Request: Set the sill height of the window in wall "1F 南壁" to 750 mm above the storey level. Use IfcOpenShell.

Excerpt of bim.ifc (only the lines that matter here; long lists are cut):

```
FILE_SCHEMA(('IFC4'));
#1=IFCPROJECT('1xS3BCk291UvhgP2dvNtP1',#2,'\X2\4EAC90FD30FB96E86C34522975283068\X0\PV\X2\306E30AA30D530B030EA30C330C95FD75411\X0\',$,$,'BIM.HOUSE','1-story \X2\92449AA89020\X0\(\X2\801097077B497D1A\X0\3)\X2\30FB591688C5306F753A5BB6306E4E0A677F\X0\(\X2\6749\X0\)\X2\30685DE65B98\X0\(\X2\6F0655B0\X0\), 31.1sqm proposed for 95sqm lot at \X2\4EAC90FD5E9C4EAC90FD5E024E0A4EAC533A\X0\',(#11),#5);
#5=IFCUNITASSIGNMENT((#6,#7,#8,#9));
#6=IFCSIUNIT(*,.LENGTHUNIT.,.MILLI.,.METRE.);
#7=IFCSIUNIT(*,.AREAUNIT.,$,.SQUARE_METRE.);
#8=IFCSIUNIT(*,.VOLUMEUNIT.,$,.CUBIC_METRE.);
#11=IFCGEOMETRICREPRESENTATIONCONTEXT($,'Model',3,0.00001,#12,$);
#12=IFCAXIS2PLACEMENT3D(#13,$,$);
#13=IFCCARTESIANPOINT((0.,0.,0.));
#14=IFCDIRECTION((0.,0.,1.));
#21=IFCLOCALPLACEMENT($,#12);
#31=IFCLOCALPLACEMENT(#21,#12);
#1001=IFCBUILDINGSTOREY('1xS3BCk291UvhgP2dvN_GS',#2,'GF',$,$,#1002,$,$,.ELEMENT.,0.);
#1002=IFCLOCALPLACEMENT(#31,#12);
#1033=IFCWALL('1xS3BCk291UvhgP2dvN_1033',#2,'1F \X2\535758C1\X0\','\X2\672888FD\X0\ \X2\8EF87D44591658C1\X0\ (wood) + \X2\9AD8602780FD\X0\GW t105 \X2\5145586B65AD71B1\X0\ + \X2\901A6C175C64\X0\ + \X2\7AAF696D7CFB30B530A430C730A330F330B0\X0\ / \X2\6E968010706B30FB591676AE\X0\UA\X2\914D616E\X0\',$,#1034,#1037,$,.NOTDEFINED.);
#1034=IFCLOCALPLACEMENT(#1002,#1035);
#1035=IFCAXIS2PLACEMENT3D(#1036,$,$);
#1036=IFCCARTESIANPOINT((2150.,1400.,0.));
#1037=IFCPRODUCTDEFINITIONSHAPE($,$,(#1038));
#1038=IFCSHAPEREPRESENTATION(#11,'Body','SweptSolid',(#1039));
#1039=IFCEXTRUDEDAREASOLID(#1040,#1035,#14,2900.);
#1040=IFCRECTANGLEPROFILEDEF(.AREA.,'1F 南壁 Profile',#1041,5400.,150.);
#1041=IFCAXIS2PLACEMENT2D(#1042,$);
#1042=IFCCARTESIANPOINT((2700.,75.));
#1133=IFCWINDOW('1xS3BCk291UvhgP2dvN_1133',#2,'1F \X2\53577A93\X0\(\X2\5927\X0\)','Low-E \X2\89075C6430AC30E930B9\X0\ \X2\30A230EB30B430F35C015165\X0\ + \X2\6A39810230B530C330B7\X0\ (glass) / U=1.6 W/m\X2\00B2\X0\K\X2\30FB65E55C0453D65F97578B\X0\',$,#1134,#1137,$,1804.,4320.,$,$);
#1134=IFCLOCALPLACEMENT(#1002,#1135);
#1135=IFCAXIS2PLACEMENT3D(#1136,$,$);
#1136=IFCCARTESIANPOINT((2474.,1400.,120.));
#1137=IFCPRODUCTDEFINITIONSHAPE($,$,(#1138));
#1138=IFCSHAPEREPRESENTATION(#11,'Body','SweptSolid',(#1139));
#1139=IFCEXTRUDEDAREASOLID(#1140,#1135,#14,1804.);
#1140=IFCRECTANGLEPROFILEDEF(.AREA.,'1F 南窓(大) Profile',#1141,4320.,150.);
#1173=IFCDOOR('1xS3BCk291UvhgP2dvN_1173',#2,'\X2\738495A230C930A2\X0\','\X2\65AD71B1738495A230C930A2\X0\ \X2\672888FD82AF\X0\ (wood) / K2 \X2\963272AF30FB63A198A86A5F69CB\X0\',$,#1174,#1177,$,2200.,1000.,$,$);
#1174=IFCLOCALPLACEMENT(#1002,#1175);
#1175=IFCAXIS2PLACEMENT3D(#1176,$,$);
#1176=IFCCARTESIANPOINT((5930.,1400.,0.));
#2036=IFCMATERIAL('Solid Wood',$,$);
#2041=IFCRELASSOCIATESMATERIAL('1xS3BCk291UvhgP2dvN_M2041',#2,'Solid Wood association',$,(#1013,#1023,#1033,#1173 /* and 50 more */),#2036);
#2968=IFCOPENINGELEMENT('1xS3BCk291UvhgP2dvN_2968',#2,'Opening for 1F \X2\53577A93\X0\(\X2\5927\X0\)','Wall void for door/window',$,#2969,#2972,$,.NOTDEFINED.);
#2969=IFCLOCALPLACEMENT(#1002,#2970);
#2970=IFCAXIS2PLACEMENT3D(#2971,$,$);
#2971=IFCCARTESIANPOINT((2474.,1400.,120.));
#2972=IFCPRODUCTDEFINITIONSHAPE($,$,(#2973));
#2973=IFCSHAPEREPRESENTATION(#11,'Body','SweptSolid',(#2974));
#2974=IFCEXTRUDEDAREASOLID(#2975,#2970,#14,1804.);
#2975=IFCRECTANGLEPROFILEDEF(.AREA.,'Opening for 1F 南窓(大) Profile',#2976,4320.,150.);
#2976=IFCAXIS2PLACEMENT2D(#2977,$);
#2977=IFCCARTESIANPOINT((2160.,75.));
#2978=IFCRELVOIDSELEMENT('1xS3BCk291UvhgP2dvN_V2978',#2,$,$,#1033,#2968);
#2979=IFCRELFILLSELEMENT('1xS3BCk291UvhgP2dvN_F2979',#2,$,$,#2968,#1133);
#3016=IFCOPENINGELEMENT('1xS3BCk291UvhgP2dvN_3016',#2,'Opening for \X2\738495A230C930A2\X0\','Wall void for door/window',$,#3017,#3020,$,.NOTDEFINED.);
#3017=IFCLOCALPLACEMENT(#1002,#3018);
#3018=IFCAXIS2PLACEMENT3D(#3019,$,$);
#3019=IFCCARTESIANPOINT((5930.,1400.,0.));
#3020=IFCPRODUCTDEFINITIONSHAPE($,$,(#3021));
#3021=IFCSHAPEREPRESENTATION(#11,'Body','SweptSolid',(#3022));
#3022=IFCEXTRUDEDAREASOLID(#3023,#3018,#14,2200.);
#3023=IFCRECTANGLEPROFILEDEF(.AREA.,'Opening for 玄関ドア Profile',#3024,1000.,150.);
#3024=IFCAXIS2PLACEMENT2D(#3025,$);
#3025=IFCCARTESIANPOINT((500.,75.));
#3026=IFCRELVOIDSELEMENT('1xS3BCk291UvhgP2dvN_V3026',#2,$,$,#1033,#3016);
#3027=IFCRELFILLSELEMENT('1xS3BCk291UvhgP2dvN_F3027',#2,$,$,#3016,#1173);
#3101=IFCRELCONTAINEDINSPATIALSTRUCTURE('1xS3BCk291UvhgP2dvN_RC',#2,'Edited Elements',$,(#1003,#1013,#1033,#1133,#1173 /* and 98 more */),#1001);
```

```python
import numpy as np
import ifcopenshell
import ifcopenshell.api.geometry
import ifcopenshell.geom
import ifcopenshell.util.element
import ifcopenshell.util.placement
import ifcopenshell.util.shape
import ifcopenshell.util.unit

model = ifcopenshell.open("bim.ifc")
unit_scale = ifcopenshell.util.unit.calculate_unit_scale(model)

window = model.by_id(1133)
opening = window.FillsVoids[0].RelatingOpeningElement
storey = ifcopenshell.util.element.get_container(window, ifc_class="IfcBuildingStorey")
level = ifcopenshell.util.placement.get_local_placement(storey.ObjectPlacement)[2, 3]

# The opening's origin need not be at the sill, so measure its lowest point.
shape = ifcopenshell.geom.create_shape(ifcopenshell.geom.settings(), opening)
bottom = ifcopenshell.util.shape.get_shape_bottom_elevation(shape, shape.geometry) / unit_scale
dz = level + 0.75 / unit_scale - bottom

shift = np.array([0.0, 0.0, dz])
# The window is not placed relative to its opening, so move both.
for product in (opening, window):
    matrix = ifcopenshell.util.placement.get_local_placement(product.ObjectPlacement)
    matrix[:3, 3] += shift
    ifcopenshell.api.geometry.edit_object_placement(model, product=product, matrix=matrix, is_si=False)

print(f"moved by {dz * unit_scale:+.3f} m")

model.write("bim-out.ifc")
```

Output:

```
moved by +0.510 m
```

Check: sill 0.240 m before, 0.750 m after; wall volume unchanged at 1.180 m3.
